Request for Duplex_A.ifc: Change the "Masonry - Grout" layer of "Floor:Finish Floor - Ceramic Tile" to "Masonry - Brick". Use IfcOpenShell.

First a look at what the model holds.

```python
import ifcopenshell
import ifcopenshell.util.element

model = ifcopenshell.open("Duplex_A.ifc")
print(model.schema)
for layer_set in model.by_type("IfcMaterialLayerSet"):
    if layer_set.LayerSetName == "Floor:Finish Floor - Ceramic Tile":
        for layer in layer_set.MaterialLayers:
            print(layer.id(), layer.Material and layer.Material.Name, layer.LayerThickness, sep=" | ")
        print(len(ifcopenshell.util.element.get_elements_by_material(model, layer_set)), "elements and types use it")
print(sorted(m.Name for m in model.by_type("IfcMaterial") if m.Name)[:60])
```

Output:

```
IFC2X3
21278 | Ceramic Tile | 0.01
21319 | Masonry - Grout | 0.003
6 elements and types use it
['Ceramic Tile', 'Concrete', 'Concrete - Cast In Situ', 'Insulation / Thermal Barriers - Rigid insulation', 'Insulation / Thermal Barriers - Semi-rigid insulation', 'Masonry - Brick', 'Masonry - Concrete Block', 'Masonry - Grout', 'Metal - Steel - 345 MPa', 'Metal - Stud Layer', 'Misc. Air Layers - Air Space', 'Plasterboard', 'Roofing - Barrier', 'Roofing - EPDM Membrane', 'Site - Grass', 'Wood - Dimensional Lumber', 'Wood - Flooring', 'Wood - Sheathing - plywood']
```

```python
import ifcopenshell
import ifcopenshell.api.material

model = ifcopenshell.open("Duplex_A.ifc")

layer_set = next(s for s in model.by_type("IfcMaterialLayerSet") if s.LayerSetName == "Floor:Finish Floor - Ceramic Tile")
layer = next(l for l in layer_set.MaterialLayers if l.Material and l.Material.Name == "Masonry - Grout")
material = next(m for m in model.by_type("IfcMaterial") if m.Name == "Masonry - Brick")

# Point this one layer at the other material; renaming the old one would change it everywhere.
ifcopenshell.api.material.edit_layer(model, layer=layer, attributes={}, material=material)

print([l.Material.Name if l.Material else None for l in layer_set.MaterialLayers])

model.write("Duplex_A-out.ifc")
```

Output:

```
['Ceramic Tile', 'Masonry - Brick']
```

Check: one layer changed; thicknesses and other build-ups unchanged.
